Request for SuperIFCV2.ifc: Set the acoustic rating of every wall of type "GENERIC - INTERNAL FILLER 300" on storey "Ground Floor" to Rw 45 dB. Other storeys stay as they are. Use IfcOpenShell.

First a look at what the model holds.

```python
import ifcopenshell
import ifcopenshell.util.element

model = ifcopenshell.open("SuperIFCV2.ifc")
print(model.schema)
storey = next(s for s in model.by_type("IfcBuildingStorey") if s.Name == "Ground Floor")
walls = [e for e in ifcopenshell.util.element.get_decomposition(storey) if e.is_a("IfcWall")]
seen = {}
for e in walls:
    element_type = ifcopenshell.util.element.get_type(e)
    key = (element_type.Name if element_type != e and element_type else None, ifcopenshell.util.element.get_pset(e, "Pset_WallCommon", "AcousticRating"))
    seen[key] = seen.get(key, 0) + 1
for (name, value), count in sorted(seen.items(), key=str):
    print(count, "x", name, "|", value)
```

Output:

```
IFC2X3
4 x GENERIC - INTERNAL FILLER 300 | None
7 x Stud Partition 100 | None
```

```python
import ifcopenshell
import ifcopenshell.api.pset
import ifcopenshell.util.element

model = ifcopenshell.open("SuperIFCV2.ifc")

storey = next(s for s in model.by_type("IfcBuildingStorey") if s.Name == "Ground Floor")
walls = [e for e in ifcopenshell.util.element.get_decomposition(storey) if e.is_a("IfcWall")]

count = 0
for e in walls:
    element_type = ifcopenshell.util.element.get_type(e)
    if element_type in (None, e) or element_type.Name != "GENERIC - INTERNAL FILLER 300":
        continue
    # add_pset returns the element's existing set when there is one.
    pset = ifcopenshell.api.pset.add_pset(model, product=e, name="Pset_WallCommon")
    ifcopenshell.api.pset.edit_pset(model, pset=pset, properties={"AcousticRating": "Rw 45 dB"})
    count += 1

print(count, "walls updated")

model.write("SuperIFCV2-out.ifc")
```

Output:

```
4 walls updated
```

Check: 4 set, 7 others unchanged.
